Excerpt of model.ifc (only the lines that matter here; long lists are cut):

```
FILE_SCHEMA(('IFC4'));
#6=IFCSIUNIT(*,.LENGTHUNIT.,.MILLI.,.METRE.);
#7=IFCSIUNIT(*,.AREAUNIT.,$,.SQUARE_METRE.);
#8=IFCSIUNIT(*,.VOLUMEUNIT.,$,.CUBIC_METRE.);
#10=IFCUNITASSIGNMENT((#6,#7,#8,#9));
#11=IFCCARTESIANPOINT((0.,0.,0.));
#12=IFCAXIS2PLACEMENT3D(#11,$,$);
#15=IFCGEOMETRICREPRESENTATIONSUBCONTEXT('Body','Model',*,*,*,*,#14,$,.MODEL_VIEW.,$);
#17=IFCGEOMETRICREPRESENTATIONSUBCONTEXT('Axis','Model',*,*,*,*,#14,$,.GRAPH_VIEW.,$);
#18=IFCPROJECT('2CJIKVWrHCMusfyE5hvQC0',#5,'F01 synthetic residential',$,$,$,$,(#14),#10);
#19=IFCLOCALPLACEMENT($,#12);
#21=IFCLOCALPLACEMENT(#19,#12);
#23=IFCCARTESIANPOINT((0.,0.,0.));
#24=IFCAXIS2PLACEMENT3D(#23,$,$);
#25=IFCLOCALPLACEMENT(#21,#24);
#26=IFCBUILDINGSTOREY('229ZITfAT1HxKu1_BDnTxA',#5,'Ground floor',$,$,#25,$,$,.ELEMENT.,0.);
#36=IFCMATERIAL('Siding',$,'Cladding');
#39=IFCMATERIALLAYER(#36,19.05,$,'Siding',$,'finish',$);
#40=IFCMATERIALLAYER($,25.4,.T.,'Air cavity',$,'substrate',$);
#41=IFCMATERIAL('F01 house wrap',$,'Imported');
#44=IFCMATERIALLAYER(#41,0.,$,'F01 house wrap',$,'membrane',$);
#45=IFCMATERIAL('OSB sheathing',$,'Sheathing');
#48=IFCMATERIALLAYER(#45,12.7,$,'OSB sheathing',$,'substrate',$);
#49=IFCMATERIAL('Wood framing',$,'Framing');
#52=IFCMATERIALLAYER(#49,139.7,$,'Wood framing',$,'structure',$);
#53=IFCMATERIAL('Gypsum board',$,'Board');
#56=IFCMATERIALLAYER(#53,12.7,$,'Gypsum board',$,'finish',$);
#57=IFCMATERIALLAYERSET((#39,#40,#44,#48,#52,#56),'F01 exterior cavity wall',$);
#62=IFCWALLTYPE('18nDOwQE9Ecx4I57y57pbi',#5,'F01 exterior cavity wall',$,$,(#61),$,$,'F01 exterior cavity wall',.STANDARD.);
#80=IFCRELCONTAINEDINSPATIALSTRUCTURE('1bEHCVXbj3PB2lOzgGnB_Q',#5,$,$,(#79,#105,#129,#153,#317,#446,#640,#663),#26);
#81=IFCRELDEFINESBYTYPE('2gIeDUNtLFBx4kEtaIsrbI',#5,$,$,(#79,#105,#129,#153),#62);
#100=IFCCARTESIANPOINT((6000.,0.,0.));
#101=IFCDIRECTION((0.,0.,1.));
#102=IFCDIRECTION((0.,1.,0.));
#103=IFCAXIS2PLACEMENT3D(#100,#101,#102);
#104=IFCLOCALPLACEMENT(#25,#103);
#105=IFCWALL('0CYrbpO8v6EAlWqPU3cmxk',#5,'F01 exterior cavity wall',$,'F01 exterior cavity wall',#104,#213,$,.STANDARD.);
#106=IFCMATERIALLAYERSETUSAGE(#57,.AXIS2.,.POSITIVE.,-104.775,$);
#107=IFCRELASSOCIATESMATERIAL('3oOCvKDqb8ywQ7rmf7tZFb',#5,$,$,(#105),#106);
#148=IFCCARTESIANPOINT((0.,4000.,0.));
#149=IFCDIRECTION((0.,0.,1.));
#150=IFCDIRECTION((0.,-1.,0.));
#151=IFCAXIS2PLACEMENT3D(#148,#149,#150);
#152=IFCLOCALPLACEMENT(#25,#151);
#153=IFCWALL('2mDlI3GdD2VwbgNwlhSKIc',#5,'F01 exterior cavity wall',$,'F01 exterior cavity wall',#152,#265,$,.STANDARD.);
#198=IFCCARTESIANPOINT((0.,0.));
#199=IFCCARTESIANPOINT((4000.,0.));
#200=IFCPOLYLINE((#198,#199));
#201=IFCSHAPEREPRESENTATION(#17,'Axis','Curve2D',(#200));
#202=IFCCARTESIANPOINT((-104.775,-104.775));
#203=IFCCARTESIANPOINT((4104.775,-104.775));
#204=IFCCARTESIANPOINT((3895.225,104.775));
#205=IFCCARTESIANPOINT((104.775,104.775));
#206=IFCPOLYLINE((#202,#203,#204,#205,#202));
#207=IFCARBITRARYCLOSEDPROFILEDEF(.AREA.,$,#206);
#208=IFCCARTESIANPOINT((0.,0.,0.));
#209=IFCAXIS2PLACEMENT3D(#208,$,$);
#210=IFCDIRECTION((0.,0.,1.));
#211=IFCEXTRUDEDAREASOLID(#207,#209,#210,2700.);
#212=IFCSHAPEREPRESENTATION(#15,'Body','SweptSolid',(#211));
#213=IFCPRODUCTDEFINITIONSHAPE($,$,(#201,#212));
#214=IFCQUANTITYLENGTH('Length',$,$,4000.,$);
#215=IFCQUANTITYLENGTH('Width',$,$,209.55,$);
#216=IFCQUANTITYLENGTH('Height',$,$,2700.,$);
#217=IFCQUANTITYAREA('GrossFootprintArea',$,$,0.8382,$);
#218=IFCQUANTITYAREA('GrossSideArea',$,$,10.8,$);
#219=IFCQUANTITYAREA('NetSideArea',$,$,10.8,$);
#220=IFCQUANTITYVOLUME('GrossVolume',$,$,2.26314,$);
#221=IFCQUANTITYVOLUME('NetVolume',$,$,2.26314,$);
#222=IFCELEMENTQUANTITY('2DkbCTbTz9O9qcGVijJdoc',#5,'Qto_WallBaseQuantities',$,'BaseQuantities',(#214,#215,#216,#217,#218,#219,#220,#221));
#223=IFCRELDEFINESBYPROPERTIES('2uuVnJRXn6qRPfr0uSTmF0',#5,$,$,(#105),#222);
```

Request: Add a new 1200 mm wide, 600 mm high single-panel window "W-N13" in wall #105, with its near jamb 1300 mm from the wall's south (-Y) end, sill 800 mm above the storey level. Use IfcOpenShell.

```python
import numpy as np
import ifcopenshell
import ifcopenshell.api.feature
import ifcopenshell.api.geometry
import ifcopenshell.api.pset
import ifcopenshell.api.root
import ifcopenshell.api.spatial
import ifcopenshell.geom
import ifcopenshell.util.element
import ifcopenshell.util.placement
import ifcopenshell.util.representation
import ifcopenshell.util.shape
import ifcopenshell.util.unit

model = ifcopenshell.open("model.ifc")
unit_scale = ifcopenshell.util.unit.calculate_unit_scale(model)
area_scale = ifcopenshell.util.unit.calculate_unit_scale(model, "AREAUNIT")
volume_scale = ifcopenshell.util.unit.calculate_unit_scale(model, "VOLUMEUNIT")
settings = ifcopenshell.geom.settings()


def volume(element):
    """Net volume in cubic metres, openings subtracted."""
    shape = ifcopenshell.geom.create_shape(settings, element)
    return ifcopenshell.util.shape.get_volume(shape.geometry)


wall = model.by_guid("0CYrbpO8v6EAlWqPU3cmxk")
storey = ifcopenshell.util.element.get_container(wall, ifc_class="IfcBuildingStorey")
context = ifcopenshell.util.representation.get_context(model, "Model", "Body", "MODEL_VIEW")
before = volume(wall)

width, height, from_end, sill = 1.2, 0.6, 1.3, 0.8  # metres

# The wall runs along its own X axis, and the end named is its -X end.
wall_shape = ifcopenshell.geom.create_shape(settings, wall)
x, y, z = ifcopenshell.util.shape.get_vertices(wall_shape.geometry).T
start = x.min() + from_end
face, thickness = float(y.min()), float(y.max() - y.min())
wall_matrix = ifcopenshell.util.placement.get_local_placement(wall.ObjectPlacement)
level = ifcopenshell.util.placement.get_local_placement(storey.ObjectPlacement)[2, 3]


def in_wall(x, y):
    """Placement at x, y metres in the wall's axes, at sill height."""
    matrix = wall_matrix.copy()
    matrix[:, 3] = wall_matrix @ np.array([x / unit_scale, y / unit_scale, 0.0, 1.0])
    matrix[2, 3] = level + sill / unit_scale
    return matrix


# Opening: a box that overshoots both wall faces by 50 mm.
opening = ifcopenshell.api.root.create_entity(model, ifc_class="IfcOpeningElement", predefined_type="OPENING")
box = ifcopenshell.api.geometry.add_wall_representation(
    model, context=context, length=width, height=height, thickness=thickness + 0.1
)
ifcopenshell.api.geometry.assign_representation(model, product=opening, representation=box)
ifcopenshell.api.geometry.edit_object_placement(model, product=opening, matrix=in_wall(start, face - 0.05), is_si=False)
ifcopenshell.api.feature.add_feature(model, feature=opening, element=wall)

window = ifcopenshell.api.root.create_entity(model, ifc_class="IfcWindow", name="W-N13", predefined_type="WINDOW")
window.OverallWidth, window.OverallHeight = width / unit_scale, height / unit_scale
window.PartitioningType = "SINGLE_PANEL"
body = ifcopenshell.api.geometry.add_window_representation(
    model,
    context=context,
    overall_width=window.OverallWidth,
    overall_height=window.OverallHeight,
    partition_type="SINGLE_PANEL",
)
ifcopenshell.api.geometry.assign_representation(model, product=window, representation=body)
ifcopenshell.api.spatial.assign_container(model, products=[window], relating_structure=storey)
ifcopenshell.api.feature.add_filling(model, opening=opening, element=window)

# Centre the window in the wall's thickness.
ifcopenshell.api.geometry.edit_object_placement(model, product=window, matrix=in_wall(start, face), is_si=False)
window_shape = ifcopenshell.geom.create_shape(settings, window)
depth = ifcopenshell.util.shape.get_vertices(window_shape.geometry)[:, 1]
offset = face + thickness / 2 - (depth.min() + depth.max()) / 2
ifcopenshell.api.geometry.edit_object_placement(model, product=window, matrix=in_wall(start, offset), is_si=False)

after = volume(wall)

# Update the wall's stored quantities.
qto = model.by_id(ifcopenshell.util.element.get_pset(wall, "Qto_WallBaseQuantities", should_inherit=False)["id"])
ifcopenshell.api.pset.edit_qto(model, qto=qto, properties={
    "NetSideArea": after / thickness / area_scale,
    "NetVolume": after / volume_scale,
})

print(f"wall volume {before:.3f} -> {after:.3f} m3")

model.write("model_updated.ifc")
```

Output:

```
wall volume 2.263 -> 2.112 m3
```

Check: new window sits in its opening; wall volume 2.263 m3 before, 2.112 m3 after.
